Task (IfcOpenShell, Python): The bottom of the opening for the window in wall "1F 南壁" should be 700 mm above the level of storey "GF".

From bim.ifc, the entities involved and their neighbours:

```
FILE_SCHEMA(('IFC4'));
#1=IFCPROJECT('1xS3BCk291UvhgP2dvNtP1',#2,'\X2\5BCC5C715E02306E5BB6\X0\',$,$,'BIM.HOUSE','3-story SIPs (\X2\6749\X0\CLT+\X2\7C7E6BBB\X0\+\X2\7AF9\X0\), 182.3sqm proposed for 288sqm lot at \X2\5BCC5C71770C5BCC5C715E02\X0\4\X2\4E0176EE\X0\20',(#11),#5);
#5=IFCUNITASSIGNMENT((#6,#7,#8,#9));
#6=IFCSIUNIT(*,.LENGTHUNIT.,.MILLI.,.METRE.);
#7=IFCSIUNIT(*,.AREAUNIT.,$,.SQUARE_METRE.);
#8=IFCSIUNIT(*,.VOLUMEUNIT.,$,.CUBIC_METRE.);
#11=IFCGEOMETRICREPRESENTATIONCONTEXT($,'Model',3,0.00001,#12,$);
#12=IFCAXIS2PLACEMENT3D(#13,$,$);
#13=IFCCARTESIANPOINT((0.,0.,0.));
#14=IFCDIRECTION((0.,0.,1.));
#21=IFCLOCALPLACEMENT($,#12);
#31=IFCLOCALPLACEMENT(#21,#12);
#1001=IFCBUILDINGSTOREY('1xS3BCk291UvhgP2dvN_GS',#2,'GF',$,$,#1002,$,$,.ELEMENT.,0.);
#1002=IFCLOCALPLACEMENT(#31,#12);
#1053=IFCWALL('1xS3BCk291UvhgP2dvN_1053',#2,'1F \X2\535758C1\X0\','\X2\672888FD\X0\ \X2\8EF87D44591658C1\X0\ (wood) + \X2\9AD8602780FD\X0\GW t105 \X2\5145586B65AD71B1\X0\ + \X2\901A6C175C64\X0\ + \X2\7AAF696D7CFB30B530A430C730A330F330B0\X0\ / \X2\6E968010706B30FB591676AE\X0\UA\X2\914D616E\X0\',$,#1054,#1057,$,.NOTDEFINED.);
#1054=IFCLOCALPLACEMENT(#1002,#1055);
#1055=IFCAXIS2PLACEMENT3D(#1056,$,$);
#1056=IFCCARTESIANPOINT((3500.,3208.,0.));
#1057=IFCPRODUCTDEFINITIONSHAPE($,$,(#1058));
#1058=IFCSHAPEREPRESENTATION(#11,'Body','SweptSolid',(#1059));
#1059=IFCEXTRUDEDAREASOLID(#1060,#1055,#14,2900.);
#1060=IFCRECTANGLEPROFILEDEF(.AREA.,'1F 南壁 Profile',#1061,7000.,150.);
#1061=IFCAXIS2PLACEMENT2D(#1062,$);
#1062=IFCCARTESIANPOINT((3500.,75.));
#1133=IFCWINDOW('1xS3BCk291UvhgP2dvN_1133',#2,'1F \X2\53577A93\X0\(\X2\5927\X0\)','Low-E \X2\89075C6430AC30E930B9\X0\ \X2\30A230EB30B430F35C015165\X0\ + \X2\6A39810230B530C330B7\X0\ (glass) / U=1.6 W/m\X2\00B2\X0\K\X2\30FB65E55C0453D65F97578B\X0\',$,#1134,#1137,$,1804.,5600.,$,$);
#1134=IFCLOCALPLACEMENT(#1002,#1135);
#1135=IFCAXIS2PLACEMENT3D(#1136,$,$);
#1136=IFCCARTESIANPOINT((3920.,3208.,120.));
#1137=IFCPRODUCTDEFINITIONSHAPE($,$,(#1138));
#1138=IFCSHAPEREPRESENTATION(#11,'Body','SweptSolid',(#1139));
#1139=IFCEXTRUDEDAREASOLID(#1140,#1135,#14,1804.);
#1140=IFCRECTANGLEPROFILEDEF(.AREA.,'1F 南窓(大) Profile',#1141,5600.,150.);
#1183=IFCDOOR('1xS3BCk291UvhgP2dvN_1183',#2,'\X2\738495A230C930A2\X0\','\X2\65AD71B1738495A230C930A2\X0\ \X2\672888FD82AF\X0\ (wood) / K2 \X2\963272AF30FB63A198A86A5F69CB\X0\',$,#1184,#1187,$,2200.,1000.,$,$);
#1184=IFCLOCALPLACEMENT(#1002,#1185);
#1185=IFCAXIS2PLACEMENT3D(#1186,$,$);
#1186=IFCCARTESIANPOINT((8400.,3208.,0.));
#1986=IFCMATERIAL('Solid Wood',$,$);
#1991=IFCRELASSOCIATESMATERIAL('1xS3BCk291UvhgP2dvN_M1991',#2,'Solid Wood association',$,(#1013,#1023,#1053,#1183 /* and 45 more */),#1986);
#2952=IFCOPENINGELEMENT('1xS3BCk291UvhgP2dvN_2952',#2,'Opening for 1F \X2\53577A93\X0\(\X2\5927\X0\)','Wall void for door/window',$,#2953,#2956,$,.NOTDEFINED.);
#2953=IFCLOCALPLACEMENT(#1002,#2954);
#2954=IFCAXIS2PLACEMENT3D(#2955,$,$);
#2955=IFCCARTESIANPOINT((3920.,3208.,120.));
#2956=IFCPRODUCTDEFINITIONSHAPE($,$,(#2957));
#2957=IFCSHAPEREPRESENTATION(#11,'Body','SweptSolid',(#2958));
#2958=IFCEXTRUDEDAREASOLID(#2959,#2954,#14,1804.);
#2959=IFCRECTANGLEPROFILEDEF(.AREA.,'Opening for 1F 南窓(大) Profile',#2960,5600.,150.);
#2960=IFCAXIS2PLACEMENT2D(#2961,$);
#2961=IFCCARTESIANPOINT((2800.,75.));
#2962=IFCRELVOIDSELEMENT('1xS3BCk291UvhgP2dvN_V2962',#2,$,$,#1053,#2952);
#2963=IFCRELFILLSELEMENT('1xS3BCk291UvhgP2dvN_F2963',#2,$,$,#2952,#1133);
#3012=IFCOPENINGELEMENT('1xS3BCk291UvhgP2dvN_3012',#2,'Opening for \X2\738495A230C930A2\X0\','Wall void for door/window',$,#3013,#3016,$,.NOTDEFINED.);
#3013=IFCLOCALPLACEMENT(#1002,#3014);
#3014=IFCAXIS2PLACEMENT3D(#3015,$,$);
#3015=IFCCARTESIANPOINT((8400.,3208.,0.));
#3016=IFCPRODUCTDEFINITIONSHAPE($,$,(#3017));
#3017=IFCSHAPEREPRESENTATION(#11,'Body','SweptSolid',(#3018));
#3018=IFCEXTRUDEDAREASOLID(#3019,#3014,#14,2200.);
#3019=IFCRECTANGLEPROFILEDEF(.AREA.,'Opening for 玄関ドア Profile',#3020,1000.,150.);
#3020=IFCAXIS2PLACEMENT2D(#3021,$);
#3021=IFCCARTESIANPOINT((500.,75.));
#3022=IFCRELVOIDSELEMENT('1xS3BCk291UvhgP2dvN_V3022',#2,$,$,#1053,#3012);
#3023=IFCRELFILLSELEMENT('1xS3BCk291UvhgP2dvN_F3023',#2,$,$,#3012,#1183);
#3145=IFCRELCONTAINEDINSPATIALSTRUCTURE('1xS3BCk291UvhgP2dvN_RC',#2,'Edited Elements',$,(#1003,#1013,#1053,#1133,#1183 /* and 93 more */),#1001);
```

```python
import numpy as np
import ifcopenshell
import ifcopenshell.api.geometry
import ifcopenshell.geom
import ifcopenshell.util.element
import ifcopenshell.util.placement
import ifcopenshell.util.shape
import ifcopenshell.util.unit

model = ifcopenshell.open("bim.ifc")
unit_scale = ifcopenshell.util.unit.calculate_unit_scale(model)

window = model.by_guid("1xS3BCk291UvhgP2dvN_1133")
opening = window.FillsVoids[0].RelatingOpeningElement
storey = ifcopenshell.util.element.get_container(window, ifc_class="IfcBuildingStorey")
level = ifcopenshell.util.placement.get_local_placement(storey.ObjectPlacement)[2, 3]

# The opening's origin need not be at the sill, so measure its lowest point.
shape = ifcopenshell.geom.create_shape(ifcopenshell.geom.settings(), opening)
bottom = ifcopenshell.util.shape.get_shape_bottom_elevation(shape, shape.geometry) / unit_scale
dz = level + 700.0 - bottom

shift = np.array([0.0, 0.0, dz])
# The window is not placed relative to its opening, so move both.
for product in (opening, window):
    matrix = ifcopenshell.util.placement.get_local_placement(product.ObjectPlacement)
    matrix[:3, 3] += shift
    ifcopenshell.api.geometry.edit_object_placement(model, product=product, matrix=matrix, is_si=False)

print(f"moved by {dz * unit_scale:+.3f} m")

model.write("bim_rev.ifc")
```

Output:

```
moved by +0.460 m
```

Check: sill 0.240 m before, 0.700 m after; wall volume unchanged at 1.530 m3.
